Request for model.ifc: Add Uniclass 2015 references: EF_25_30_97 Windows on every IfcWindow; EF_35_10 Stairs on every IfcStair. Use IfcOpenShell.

First a look at what the model holds.

```python
import ifcopenshell

model = ifcopenshell.open("model.ifc")
print(model.schema)
print("classifications:", [c.Name for c in model.by_type("IfcClassification")])
for ifc_class in ("IfcDoor", "IfcRoof", "IfcStair", "IfcWall", "IfcWindow"):
    print(ifc_class, len(model.by_type(ifc_class)))
```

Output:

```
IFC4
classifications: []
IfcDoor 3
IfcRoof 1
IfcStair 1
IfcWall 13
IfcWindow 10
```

```python
import ifcopenshell
import ifcopenshell.api.classification

model = ifcopenshell.open("model.ifc")

system = ifcopenshell.api.classification.add_classification(model, classification="Uniclass 2015")

codes = {
    "IfcWindow": ("EF_25_30_97", "Windows"),
    "IfcStair": ("EF_35_10", "Stairs"),
}
for ifc_class, (code, name) in codes.items():
    products = model.by_type(ifc_class)
    ifcopenshell.api.classification.add_reference(
        model, products=products, classification=system, identification=code, name=name
    )
    print(code, len(products))

model.write("model_updated.ifc")
```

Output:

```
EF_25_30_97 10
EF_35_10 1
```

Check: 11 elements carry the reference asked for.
